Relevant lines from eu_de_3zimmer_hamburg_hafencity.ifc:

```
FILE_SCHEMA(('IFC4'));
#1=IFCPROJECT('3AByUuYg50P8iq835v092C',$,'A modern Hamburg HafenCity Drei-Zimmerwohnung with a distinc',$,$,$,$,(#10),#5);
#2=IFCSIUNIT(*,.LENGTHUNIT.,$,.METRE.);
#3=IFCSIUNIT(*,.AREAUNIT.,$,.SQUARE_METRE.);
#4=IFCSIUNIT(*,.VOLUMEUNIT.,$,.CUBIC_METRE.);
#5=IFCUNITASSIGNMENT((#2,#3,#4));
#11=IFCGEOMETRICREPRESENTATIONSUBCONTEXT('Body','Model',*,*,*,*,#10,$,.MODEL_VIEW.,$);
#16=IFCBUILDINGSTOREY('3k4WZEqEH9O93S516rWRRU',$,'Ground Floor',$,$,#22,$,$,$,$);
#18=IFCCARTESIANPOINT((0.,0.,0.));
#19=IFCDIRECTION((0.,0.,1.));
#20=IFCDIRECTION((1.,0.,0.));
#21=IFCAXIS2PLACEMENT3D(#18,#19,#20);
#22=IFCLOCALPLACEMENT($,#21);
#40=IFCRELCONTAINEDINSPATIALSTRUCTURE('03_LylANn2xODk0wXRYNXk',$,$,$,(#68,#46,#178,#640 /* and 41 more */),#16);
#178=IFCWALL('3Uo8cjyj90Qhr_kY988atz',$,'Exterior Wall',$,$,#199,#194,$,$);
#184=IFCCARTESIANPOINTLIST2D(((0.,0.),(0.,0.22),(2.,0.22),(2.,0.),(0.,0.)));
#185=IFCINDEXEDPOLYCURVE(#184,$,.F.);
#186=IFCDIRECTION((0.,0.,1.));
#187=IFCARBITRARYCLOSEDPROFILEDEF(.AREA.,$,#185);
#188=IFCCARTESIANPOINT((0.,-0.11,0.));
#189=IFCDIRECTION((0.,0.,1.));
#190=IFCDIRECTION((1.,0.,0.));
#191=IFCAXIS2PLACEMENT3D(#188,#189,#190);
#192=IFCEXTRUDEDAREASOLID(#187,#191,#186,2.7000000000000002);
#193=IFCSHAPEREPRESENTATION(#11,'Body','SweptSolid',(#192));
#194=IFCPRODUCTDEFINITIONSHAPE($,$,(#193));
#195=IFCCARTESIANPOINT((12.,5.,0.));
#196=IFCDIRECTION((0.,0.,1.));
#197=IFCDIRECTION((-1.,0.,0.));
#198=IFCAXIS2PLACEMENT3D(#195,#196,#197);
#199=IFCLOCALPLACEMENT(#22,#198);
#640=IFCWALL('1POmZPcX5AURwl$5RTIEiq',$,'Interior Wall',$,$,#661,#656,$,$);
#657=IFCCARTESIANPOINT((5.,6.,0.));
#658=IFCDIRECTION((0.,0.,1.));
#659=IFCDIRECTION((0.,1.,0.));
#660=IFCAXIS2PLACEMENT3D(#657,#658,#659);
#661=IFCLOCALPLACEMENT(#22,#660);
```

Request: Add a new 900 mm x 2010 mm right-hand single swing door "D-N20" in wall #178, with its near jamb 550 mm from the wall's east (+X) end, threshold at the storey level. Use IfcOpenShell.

```python
import numpy as np
import ifcopenshell
import ifcopenshell.api.feature
import ifcopenshell.api.geometry
import ifcopenshell.api.root
import ifcopenshell.api.spatial
import ifcopenshell.geom
import ifcopenshell.util.element
import ifcopenshell.util.placement
import ifcopenshell.util.representation
import ifcopenshell.util.shape
import ifcopenshell.util.unit

model = ifcopenshell.open("eu_de_3zimmer_hamburg_hafencity.ifc")
unit_scale = ifcopenshell.util.unit.calculate_unit_scale(model)
settings = ifcopenshell.geom.settings()


def volume(element):
    """Net volume in cubic metres, openings subtracted."""
    shape = ifcopenshell.geom.create_shape(settings, element)
    return ifcopenshell.util.shape.get_volume(shape.geometry)


wall = model.by_guid("3Uo8cjyj90Qhr_kY988atz")
storey = ifcopenshell.util.element.get_container(wall, ifc_class="IfcBuildingStorey")
context = ifcopenshell.util.representation.get_context(model, "Model", "Body", "MODEL_VIEW")
before = volume(wall)

width, height, from_end, sill = 0.9, 2.01, 0.55, 0.0  # metres

# The wall runs along its own X axis, and the end named is its -X end.
wall_shape = ifcopenshell.geom.create_shape(settings, wall)
x, y, z = ifcopenshell.util.shape.get_vertices(wall_shape.geometry).T
start = x.min() + from_end
face, thickness = float(y.min()), float(y.max() - y.min())
wall_matrix = ifcopenshell.util.placement.get_local_placement(wall.ObjectPlacement)
level = ifcopenshell.util.placement.get_local_placement(storey.ObjectPlacement)[2, 3]


def in_wall(x, y):
    """Placement at x, y metres in the wall's axes, at sill height."""
    matrix = wall_matrix.copy()
    matrix[:, 3] = wall_matrix @ np.array([x / unit_scale, y / unit_scale, 0.0, 1.0])
    matrix[2, 3] = level + sill / unit_scale
    return matrix


# Opening: a box that overshoots both wall faces by 50 mm.
opening = ifcopenshell.api.root.create_entity(model, ifc_class="IfcOpeningElement", predefined_type="OPENING")
box = ifcopenshell.api.geometry.add_wall_representation(
    model, context=context, length=width, height=height, thickness=thickness + 0.1
)
ifcopenshell.api.geometry.assign_representation(model, product=opening, representation=box)
ifcopenshell.api.geometry.edit_object_placement(model, product=opening, matrix=in_wall(start, face - 0.05), is_si=False)
ifcopenshell.api.feature.add_feature(model, feature=opening, element=wall)

door = ifcopenshell.api.root.create_entity(model, ifc_class="IfcDoor", name="D-N20", predefined_type="DOOR")
door.OverallWidth, door.OverallHeight = width / unit_scale, height / unit_scale
door.OperationType = "SINGLE_SWING_RIGHT"
body = ifcopenshell.api.geometry.add_door_representation(
    model,
    context=context,
    overall_width=door.OverallWidth,
    overall_height=door.OverallHeight,
    operation_type="SINGLE_SWING_RIGHT",
    lining_properties={"LiningDepth": thickness / unit_scale, "ThresholdDepth": thickness / unit_scale},
)
ifcopenshell.api.geometry.assign_representation(model, product=door, representation=body)
ifcopenshell.api.spatial.assign_container(model, products=[door], relating_structure=storey)
ifcopenshell.api.feature.add_filling(model, opening=opening, element=door)

# The lining spans the wall, so the door starts at the wall face.
ifcopenshell.api.geometry.edit_object_placement(model, product=door, matrix=in_wall(start, face), is_si=False)

after = volume(wall)

print(f"wall volume {before:.3f} -> {after:.3f} m3")

model.write("eu_de_3zimmer_hamburg_hafencity_rev.ifc")
```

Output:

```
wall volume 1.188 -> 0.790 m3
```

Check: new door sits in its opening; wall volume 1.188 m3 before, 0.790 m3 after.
